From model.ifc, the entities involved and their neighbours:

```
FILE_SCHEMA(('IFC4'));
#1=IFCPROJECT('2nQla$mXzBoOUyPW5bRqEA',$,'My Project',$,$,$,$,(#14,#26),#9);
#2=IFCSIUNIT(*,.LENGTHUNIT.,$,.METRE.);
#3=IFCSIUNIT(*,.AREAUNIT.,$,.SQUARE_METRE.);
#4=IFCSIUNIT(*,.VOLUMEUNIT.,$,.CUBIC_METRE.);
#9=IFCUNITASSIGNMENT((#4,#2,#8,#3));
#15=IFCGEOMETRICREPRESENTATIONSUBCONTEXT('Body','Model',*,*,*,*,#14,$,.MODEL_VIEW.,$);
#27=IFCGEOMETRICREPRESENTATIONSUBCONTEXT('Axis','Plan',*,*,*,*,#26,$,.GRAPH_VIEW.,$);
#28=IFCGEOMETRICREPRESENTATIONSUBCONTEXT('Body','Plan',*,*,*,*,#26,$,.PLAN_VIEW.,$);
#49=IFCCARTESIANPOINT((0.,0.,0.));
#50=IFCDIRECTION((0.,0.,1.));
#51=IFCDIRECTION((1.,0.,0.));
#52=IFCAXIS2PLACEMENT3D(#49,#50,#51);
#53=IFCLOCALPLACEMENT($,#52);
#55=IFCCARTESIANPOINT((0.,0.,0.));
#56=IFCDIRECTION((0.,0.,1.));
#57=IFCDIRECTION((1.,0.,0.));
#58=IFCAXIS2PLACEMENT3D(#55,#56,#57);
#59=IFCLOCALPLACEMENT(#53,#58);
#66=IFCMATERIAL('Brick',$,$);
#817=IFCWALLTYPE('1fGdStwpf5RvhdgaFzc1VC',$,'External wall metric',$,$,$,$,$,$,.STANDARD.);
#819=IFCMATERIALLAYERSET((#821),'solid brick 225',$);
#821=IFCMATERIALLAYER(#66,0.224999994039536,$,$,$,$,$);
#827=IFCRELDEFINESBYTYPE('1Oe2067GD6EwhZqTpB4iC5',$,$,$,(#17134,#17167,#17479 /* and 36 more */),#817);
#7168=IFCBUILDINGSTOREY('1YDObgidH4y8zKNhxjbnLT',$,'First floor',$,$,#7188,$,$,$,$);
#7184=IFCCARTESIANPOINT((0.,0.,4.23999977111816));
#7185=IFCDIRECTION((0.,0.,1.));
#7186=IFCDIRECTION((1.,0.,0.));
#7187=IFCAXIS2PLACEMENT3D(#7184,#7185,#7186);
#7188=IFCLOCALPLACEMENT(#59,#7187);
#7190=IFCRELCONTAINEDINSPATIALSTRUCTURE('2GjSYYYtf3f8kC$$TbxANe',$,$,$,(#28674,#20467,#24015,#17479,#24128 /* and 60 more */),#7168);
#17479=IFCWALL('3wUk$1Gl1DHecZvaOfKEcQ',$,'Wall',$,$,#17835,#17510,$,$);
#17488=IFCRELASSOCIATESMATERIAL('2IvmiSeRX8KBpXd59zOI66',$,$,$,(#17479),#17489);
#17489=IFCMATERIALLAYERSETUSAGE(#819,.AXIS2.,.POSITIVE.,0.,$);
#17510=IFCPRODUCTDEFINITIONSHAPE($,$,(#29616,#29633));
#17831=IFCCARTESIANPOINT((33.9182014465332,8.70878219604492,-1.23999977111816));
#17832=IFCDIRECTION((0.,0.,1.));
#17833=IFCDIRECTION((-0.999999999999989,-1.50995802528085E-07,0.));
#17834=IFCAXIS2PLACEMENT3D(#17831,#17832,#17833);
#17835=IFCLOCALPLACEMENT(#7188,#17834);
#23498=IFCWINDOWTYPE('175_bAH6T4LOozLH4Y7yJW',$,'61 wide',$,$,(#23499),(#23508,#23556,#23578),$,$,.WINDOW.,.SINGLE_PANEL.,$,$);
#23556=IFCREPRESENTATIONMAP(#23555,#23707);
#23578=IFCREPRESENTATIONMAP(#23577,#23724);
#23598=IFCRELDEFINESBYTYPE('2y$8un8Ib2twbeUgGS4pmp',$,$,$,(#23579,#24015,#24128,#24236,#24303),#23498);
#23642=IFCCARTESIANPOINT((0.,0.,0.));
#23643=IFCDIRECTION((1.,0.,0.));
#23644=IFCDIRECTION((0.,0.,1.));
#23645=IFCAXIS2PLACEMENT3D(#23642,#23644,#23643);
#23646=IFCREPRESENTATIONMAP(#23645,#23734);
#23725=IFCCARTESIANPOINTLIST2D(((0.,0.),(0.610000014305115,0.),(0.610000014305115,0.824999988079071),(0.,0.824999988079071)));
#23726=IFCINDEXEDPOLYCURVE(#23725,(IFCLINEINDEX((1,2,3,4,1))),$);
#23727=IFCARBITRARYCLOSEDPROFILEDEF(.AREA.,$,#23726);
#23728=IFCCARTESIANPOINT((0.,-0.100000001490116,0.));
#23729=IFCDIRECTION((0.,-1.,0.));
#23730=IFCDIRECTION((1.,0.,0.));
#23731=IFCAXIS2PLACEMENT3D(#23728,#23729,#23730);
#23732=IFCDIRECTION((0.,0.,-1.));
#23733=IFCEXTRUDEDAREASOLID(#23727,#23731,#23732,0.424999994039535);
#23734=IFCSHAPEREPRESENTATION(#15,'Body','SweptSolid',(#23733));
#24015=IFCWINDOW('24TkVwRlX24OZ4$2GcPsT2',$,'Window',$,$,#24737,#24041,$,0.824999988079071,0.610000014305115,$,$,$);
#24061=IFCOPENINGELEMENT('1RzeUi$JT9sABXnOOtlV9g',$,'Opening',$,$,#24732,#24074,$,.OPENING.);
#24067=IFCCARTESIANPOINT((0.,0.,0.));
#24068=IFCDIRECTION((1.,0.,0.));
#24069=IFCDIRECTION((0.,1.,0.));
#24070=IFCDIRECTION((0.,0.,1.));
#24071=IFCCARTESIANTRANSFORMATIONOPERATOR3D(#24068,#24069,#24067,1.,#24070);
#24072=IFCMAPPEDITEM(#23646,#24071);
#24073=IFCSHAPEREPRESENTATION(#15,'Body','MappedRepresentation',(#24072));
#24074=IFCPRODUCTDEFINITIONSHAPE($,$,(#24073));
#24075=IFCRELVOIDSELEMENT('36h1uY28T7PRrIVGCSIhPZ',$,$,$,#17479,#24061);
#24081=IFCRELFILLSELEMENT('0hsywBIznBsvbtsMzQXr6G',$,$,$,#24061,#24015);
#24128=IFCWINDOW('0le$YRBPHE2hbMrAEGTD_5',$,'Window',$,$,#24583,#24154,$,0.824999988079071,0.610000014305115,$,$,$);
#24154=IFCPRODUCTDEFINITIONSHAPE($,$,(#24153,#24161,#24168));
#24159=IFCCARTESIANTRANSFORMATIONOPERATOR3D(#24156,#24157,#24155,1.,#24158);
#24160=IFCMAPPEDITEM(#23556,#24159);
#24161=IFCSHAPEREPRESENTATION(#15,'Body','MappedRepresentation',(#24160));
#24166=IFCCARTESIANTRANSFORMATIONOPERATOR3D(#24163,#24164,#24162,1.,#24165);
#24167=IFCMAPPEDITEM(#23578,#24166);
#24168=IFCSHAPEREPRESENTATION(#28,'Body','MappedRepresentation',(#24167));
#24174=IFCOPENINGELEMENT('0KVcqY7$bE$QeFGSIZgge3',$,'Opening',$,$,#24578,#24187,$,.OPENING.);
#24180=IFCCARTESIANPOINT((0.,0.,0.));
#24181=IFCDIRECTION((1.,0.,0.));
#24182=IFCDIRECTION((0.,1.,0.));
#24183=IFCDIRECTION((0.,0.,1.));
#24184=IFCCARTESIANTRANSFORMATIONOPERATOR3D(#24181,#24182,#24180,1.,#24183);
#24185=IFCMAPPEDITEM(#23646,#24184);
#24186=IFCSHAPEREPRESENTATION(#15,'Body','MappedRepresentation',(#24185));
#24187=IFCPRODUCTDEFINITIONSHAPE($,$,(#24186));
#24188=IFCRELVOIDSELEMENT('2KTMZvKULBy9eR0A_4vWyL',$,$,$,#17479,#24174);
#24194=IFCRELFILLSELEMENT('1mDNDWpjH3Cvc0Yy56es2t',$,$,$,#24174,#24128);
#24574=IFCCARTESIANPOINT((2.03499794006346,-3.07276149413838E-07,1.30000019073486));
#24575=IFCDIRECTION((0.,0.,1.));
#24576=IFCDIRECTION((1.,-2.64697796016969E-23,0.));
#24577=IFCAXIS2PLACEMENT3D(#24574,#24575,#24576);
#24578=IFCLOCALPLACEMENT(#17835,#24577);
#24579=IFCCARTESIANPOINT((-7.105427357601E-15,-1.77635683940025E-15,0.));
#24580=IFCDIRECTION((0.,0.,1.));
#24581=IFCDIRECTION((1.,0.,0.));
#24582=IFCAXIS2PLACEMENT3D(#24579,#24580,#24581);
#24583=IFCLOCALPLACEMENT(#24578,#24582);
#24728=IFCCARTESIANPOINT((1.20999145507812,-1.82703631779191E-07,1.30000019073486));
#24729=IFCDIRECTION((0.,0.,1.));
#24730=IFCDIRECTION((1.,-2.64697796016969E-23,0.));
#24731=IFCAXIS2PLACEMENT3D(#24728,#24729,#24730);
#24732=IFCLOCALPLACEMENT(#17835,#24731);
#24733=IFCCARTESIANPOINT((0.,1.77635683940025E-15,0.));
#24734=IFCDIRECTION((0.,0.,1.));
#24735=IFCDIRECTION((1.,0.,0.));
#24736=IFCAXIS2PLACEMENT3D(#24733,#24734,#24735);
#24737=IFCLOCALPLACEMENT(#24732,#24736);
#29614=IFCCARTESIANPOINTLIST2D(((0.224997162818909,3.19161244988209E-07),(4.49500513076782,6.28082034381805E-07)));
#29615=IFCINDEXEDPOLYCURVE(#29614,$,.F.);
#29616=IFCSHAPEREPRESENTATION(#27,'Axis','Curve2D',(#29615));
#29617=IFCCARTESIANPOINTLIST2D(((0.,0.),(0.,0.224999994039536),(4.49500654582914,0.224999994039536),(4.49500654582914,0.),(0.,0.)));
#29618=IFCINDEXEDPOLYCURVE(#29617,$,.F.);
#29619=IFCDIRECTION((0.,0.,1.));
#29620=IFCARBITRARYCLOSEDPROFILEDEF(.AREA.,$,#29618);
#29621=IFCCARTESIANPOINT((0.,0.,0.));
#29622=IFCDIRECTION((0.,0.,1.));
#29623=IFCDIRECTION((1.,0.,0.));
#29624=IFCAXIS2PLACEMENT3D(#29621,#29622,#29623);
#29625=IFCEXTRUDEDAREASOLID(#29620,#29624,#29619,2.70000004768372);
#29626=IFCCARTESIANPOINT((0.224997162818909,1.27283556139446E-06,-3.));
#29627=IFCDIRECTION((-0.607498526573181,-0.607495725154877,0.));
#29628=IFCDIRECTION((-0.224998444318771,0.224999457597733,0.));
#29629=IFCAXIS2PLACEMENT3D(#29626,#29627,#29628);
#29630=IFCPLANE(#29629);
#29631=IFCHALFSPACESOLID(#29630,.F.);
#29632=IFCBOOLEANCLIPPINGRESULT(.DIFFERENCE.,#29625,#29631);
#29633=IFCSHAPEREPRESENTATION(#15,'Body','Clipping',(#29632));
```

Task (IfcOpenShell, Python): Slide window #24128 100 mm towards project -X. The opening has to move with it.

```python
import ifcopenshell
import ifcopenshell.api.geometry
import ifcopenshell.util.placement

model = ifcopenshell.open("model.ifc")

window = model.by_guid("0le$YRBPHE2hbMrAEGTD_5")
opening = window.FillsVoids[0].RelatingOpeningElement
wall = opening.VoidsElements[0].RelatingBuildingElement

wall_matrix = ifcopenshell.util.placement.get_local_placement(wall.ObjectPlacement)
shift = wall_matrix[:3, 0] * 0.1
before = ifcopenshell.util.placement.get_local_placement(window.ObjectPlacement)[:3, 3].copy()

# The window is placed relative to its opening, so it follows when the opening moves.
matrix = ifcopenshell.util.placement.get_local_placement(opening.ObjectPlacement)
matrix[:3, 3] += shift
ifcopenshell.api.geometry.edit_object_placement(
    model, product=opening, matrix=matrix, is_si=False, should_transform_children=True
)

after = ifcopenshell.util.placement.get_local_placement(window.ObjectPlacement)[:3, 3]
print("window moved by", (after - before).round(3) + 0.0)

model.write("model_rev.ifc")
```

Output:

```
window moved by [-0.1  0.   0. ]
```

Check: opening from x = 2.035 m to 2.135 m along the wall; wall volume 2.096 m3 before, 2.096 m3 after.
